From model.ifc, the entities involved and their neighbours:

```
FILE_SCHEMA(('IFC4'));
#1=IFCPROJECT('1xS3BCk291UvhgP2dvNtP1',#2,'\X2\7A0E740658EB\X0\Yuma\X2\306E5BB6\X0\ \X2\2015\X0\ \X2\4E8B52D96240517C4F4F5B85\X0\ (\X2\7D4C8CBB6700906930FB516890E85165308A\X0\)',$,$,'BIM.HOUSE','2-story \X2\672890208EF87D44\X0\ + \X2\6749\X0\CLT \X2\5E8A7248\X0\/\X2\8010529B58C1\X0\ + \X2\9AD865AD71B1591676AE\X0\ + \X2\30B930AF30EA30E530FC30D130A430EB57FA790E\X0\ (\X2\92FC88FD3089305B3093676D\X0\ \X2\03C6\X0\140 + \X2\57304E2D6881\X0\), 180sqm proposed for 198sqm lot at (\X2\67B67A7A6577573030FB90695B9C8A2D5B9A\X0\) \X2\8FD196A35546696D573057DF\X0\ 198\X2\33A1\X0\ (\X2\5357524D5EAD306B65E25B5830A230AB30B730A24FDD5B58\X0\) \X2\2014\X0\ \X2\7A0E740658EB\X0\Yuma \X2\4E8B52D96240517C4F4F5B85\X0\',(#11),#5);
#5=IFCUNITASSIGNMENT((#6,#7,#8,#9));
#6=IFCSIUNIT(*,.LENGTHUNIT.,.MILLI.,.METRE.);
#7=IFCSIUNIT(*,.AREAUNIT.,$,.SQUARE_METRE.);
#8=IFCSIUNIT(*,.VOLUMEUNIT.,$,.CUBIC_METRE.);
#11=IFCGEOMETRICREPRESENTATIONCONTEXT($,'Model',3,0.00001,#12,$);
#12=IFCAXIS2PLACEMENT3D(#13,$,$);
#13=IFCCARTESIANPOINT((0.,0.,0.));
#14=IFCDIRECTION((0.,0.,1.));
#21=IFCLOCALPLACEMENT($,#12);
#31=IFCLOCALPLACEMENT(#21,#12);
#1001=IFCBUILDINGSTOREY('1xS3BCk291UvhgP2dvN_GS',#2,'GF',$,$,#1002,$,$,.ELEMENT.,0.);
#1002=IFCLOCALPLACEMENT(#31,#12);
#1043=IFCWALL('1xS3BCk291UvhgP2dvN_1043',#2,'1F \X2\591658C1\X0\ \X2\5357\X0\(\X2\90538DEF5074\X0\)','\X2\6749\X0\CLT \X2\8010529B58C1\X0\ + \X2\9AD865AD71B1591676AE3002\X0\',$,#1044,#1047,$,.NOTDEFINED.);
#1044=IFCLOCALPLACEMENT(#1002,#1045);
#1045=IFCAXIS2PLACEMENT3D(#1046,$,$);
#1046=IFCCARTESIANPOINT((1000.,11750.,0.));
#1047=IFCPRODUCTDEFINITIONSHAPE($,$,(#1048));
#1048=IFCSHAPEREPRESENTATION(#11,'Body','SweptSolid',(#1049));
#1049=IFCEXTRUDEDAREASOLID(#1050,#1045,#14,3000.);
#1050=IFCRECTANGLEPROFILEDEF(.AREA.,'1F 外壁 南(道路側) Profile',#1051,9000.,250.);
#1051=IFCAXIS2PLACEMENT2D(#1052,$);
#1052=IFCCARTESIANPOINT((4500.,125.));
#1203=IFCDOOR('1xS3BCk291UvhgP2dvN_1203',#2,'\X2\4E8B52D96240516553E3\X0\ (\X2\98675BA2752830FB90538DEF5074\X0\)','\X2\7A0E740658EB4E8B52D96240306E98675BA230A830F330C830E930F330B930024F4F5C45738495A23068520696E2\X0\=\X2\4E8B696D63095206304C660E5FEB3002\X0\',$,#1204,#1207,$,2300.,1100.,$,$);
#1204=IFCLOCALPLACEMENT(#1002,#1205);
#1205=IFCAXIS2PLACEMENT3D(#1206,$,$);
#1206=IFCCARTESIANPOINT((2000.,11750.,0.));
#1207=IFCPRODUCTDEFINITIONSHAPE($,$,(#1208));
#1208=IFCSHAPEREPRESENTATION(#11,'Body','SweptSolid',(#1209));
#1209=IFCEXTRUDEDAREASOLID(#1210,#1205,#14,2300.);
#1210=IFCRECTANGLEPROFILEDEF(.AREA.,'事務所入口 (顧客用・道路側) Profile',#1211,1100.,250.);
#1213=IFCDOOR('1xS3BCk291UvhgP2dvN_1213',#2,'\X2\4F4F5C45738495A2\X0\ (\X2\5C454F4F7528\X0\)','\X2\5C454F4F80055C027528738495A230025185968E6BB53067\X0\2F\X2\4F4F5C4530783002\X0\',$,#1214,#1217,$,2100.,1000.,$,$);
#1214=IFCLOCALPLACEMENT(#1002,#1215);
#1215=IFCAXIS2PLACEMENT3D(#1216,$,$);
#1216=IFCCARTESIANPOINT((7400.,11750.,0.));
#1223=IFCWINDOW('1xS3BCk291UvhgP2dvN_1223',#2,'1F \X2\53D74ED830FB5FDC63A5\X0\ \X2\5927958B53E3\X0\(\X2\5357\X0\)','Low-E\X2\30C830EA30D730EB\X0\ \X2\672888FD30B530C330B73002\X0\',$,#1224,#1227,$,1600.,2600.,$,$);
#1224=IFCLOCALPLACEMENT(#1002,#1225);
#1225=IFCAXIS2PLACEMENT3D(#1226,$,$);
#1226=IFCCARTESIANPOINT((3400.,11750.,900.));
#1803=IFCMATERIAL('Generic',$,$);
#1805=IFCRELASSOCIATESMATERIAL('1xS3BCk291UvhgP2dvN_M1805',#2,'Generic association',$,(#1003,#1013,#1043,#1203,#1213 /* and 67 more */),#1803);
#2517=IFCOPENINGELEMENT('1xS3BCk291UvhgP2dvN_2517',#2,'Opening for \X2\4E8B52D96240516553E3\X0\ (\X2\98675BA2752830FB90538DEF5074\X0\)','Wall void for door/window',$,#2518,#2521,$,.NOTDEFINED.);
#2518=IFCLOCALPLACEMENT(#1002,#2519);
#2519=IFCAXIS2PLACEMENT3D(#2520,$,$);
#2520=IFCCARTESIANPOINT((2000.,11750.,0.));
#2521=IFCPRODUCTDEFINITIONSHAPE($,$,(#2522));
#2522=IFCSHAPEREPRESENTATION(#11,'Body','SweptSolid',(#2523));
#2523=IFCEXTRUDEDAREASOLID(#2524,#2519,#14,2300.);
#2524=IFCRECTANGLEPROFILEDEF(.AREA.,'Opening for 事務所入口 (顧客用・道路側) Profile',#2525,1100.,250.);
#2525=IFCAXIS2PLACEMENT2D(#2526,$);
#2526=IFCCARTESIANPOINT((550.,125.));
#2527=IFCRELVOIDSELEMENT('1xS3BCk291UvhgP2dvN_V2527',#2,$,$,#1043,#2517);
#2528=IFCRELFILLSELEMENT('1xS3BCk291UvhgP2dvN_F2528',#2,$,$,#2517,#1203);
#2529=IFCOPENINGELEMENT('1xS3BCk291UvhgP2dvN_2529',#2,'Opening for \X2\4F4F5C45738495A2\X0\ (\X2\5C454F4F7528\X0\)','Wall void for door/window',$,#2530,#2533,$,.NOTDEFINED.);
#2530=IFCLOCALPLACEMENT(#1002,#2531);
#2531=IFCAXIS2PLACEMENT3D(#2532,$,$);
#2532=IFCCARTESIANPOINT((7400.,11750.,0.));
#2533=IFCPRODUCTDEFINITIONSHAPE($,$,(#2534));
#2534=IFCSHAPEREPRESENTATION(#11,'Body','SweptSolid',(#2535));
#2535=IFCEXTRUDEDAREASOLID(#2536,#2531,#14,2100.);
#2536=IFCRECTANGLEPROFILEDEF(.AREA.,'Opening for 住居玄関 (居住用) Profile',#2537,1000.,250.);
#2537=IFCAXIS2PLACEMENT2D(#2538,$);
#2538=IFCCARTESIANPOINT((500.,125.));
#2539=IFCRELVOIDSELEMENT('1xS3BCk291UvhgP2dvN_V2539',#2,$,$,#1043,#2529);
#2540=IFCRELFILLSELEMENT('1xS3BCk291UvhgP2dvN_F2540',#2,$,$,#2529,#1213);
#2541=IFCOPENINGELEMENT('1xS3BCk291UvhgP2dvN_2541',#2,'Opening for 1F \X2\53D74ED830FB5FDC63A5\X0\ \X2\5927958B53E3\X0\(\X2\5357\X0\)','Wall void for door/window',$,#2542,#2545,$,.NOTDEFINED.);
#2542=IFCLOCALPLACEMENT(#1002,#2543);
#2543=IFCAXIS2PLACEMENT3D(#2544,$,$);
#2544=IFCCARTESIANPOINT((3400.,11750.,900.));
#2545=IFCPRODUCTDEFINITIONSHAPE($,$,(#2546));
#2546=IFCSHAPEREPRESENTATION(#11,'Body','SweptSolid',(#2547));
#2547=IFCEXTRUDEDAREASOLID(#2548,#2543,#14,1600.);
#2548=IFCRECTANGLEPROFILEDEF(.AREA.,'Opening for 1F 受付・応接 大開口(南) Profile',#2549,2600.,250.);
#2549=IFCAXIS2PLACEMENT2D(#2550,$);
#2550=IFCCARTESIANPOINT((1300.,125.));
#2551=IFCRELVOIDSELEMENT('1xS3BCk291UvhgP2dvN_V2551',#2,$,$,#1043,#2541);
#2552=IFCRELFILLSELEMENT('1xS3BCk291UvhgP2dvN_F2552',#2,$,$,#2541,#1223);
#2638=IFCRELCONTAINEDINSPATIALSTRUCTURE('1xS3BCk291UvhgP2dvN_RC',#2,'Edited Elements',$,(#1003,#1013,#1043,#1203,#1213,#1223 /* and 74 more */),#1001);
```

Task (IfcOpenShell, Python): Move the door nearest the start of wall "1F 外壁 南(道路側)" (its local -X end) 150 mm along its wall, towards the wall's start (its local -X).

```python
import ifcopenshell
import ifcopenshell.api.geometry
import ifcopenshell.util.placement

model = ifcopenshell.open("model.ifc")

door = model.by_guid("1xS3BCk291UvhgP2dvN_1203")
opening = door.FillsVoids[0].RelatingOpeningElement
wall = opening.VoidsElements[0].RelatingBuildingElement

wall_matrix = ifcopenshell.util.placement.get_local_placement(wall.ObjectPlacement)
shift = wall_matrix[:3, 0] * -150.0
before = ifcopenshell.util.placement.get_local_placement(door.ObjectPlacement)[:3, 3].copy()

# The door is not placed relative to its opening, so move both.
for product in (opening, door):
    matrix = ifcopenshell.util.placement.get_local_placement(product.ObjectPlacement)
    matrix[:3, 3] += shift
    ifcopenshell.api.geometry.edit_object_placement(model, product=product, matrix=matrix, is_si=False)

after = ifcopenshell.util.placement.get_local_placement(door.ObjectPlacement)[:3, 3]
print("door moved by", (after - before).round(3) + 0.0)

model.write("model_edited.ifc")
```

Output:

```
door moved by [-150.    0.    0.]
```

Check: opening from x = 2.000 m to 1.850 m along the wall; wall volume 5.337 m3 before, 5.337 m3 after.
